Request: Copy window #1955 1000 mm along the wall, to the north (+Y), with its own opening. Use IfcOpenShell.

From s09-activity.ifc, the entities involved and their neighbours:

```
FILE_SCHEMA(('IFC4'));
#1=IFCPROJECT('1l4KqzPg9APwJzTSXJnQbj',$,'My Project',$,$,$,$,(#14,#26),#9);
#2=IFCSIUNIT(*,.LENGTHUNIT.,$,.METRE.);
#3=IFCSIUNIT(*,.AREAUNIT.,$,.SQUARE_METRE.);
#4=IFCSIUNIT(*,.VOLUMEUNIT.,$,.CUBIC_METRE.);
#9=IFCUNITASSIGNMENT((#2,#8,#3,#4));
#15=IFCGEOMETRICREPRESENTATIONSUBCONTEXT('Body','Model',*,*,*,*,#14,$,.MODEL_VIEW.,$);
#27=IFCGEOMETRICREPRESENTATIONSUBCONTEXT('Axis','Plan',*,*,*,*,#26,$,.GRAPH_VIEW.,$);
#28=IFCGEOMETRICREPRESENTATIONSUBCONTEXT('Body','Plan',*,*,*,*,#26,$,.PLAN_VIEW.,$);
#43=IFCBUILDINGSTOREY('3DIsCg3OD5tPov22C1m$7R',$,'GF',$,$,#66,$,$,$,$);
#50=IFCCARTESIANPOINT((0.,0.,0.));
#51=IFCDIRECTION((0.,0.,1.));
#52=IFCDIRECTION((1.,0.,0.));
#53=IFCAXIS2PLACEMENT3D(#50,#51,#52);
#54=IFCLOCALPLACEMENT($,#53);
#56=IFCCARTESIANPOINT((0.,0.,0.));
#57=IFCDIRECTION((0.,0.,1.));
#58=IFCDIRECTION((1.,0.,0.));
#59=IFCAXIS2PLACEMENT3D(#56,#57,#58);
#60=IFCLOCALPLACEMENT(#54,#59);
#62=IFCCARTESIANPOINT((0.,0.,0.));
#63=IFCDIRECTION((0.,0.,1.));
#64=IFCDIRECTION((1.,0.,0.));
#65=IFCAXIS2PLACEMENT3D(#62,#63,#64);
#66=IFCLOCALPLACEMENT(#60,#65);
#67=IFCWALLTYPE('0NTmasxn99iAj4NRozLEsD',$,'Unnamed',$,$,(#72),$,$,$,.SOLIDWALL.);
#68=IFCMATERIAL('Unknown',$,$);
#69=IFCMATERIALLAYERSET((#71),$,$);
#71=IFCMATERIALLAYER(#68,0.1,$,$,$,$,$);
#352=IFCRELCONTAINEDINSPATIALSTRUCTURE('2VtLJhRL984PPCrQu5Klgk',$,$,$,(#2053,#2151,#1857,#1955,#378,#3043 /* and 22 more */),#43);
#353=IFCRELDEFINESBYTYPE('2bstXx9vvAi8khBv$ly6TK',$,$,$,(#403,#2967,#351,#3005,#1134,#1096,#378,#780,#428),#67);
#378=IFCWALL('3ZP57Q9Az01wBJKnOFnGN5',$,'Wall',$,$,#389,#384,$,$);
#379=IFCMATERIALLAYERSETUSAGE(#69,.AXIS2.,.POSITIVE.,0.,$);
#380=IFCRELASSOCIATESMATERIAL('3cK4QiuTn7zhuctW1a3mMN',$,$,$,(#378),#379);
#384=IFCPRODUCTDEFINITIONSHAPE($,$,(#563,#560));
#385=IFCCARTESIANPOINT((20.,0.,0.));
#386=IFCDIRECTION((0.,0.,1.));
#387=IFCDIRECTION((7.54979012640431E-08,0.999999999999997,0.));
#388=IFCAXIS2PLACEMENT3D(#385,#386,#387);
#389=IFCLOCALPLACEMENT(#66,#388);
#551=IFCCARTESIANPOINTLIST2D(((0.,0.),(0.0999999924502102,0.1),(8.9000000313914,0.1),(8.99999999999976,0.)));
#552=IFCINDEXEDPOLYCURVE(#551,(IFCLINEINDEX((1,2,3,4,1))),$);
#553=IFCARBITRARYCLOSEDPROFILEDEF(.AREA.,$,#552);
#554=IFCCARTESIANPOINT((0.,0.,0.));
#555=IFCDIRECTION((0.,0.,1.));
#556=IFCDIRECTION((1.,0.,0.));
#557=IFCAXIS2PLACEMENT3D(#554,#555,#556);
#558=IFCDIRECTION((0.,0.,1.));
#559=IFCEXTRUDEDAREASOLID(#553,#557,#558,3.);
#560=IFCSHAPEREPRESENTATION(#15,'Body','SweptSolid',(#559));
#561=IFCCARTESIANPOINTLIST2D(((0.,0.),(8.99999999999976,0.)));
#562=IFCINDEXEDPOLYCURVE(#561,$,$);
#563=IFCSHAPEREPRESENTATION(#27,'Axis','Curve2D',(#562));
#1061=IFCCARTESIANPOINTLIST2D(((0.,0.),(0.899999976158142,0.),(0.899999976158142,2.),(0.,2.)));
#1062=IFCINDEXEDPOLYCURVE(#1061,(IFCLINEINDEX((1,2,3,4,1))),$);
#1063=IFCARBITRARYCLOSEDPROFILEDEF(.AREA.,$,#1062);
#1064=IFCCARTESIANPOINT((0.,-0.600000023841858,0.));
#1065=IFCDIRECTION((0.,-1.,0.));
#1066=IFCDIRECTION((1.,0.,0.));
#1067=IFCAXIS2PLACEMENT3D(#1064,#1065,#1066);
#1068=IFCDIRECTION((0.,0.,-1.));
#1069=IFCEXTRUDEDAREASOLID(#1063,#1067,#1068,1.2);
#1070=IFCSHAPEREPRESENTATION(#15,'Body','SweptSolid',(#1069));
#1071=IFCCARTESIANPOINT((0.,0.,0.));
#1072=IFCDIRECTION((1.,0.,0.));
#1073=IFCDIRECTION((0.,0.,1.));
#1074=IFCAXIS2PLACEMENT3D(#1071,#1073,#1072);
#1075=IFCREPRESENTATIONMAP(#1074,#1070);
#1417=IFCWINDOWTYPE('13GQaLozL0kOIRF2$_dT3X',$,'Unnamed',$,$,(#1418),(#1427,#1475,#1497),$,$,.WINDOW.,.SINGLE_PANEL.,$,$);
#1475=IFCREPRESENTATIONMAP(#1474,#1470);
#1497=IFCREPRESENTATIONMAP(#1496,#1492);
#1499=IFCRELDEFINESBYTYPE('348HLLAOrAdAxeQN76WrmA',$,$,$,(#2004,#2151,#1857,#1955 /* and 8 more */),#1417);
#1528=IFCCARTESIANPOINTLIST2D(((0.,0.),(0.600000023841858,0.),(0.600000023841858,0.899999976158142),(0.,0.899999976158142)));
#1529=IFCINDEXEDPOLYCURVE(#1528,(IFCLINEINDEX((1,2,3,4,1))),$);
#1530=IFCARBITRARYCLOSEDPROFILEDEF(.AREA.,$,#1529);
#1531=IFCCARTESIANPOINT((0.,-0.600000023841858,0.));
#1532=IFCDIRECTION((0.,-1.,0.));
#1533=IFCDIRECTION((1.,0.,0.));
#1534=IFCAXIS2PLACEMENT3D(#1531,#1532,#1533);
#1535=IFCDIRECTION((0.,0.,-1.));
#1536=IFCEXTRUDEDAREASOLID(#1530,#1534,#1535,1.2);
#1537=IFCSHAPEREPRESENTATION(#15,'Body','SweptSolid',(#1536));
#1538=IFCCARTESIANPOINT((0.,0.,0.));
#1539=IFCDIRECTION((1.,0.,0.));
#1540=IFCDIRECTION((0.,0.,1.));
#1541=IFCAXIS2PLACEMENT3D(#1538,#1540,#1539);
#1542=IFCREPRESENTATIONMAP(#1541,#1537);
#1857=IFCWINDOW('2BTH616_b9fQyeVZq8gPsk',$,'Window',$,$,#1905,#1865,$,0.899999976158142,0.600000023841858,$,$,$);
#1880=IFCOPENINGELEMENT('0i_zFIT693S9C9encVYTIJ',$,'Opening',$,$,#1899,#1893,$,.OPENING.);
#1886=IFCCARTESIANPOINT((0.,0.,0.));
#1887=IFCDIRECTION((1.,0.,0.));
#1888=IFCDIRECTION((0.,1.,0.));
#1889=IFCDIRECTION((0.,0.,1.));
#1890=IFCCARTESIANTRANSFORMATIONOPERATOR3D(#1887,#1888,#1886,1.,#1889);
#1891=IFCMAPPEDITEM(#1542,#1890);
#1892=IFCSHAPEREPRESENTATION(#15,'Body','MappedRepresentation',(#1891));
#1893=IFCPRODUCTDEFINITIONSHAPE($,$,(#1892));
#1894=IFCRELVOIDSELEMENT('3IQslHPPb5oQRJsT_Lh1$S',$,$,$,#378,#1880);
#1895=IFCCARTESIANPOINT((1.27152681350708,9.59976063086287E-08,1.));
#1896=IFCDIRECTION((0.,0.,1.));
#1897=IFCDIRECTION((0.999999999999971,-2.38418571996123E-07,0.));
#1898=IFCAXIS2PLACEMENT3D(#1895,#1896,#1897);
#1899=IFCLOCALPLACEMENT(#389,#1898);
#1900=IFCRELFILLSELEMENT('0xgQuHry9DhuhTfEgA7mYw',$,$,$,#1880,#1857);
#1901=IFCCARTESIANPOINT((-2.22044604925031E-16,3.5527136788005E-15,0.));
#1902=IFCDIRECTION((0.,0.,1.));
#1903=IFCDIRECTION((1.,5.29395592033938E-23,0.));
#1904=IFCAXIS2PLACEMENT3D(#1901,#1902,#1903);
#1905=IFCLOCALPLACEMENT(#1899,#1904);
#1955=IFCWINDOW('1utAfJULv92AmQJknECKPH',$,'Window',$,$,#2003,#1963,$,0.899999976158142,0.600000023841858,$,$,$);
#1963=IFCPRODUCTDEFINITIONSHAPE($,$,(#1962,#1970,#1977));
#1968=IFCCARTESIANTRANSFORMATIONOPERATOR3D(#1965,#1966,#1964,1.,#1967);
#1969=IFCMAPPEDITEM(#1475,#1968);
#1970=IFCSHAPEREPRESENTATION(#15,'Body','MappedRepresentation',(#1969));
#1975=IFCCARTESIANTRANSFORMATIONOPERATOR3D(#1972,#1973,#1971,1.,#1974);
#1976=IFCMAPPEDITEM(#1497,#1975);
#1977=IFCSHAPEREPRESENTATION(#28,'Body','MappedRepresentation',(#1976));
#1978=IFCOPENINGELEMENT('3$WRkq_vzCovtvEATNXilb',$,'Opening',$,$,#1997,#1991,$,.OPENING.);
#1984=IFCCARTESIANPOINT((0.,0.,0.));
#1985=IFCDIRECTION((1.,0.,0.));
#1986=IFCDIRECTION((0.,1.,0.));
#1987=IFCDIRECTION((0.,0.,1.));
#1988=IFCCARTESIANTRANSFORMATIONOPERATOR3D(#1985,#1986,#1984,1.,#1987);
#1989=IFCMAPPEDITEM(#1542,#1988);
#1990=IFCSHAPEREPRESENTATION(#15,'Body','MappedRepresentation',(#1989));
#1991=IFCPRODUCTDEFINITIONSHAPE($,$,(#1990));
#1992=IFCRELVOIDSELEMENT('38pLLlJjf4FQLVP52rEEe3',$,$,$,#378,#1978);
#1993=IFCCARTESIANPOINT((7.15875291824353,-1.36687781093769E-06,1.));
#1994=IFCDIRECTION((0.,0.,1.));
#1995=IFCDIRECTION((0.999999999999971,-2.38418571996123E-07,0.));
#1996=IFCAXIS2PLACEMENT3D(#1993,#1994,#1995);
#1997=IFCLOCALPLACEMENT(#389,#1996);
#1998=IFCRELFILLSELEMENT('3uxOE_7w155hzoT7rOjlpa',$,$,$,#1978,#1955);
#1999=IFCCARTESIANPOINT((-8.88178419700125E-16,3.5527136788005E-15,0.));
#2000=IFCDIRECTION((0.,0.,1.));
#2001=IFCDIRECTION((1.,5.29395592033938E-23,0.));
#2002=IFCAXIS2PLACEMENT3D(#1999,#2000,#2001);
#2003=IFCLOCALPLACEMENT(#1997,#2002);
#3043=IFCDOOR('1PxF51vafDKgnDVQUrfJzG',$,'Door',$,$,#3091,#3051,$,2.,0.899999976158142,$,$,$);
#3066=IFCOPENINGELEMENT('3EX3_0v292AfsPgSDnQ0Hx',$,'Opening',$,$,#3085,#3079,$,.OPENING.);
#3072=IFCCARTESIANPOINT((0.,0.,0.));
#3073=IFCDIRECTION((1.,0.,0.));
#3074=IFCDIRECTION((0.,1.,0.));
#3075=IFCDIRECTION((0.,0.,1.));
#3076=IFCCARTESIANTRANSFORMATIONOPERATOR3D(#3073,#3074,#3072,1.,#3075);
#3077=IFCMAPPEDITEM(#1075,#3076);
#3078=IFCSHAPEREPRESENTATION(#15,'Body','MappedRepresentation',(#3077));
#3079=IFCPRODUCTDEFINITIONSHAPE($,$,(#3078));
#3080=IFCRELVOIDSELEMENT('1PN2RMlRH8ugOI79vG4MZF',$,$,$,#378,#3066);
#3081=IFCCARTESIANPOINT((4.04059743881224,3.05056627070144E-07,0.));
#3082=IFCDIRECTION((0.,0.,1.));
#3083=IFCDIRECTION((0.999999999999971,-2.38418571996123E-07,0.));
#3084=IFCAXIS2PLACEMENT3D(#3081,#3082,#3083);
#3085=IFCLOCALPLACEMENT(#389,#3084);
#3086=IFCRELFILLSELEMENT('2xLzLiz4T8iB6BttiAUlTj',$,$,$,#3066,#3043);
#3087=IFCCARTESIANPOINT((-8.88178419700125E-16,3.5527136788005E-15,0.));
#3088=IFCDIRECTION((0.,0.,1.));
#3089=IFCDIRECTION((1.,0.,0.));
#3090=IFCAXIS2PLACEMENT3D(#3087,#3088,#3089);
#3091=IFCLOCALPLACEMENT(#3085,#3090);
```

```python
import ifcopenshell
import ifcopenshell.api.feature
import ifcopenshell.api.geometry
import ifcopenshell.api.root
import ifcopenshell.geom
import ifcopenshell.util.element
import ifcopenshell.util.placement
import ifcopenshell.util.shape
import ifcopenshell.util.unit

model = ifcopenshell.open("s09-activity.ifc")
unit_scale = ifcopenshell.util.unit.calculate_unit_scale(model)
settings = ifcopenshell.geom.settings()


def volume(element):
    """Net volume in cubic metres, openings subtracted."""
    shape = ifcopenshell.geom.create_shape(settings, element)
    return ifcopenshell.util.shape.get_volume(shape.geometry)


window = model.by_guid("1utAfJULv92AmQJknECKPH")
opening = window.FillsVoids[0].RelatingOpeningElement
wall = opening.VoidsElements[0].RelatingBuildingElement
before = volume(wall)
shift = ifcopenshell.util.placement.get_local_placement(wall.ObjectPlacement)[:3, 0] * 1 / unit_scale

# copy_class copies the void relationship, type, container and properties, but no geometry.
new_opening = ifcopenshell.api.root.copy_class(model, product=opening)
new_opening.Representation = ifcopenshell.util.element.copy_deep(
    model, opening.Representation, exclude=["IfcGeometricRepresentationContext", "IfcRepresentationMap"]
)
new_window = ifcopenshell.api.root.copy_class(model, product=window)
new_window.Representation = ifcopenshell.util.element.copy_deep(
    model, window.Representation, exclude=["IfcGeometricRepresentationContext", "IfcRepresentationMap"]
)
ifcopenshell.api.feature.add_filling(model, opening=new_opening, element=new_window)

for old, new in ((opening, new_opening), (window, new_window)):
    matrix = ifcopenshell.util.placement.get_local_placement(old.ObjectPlacement)
    matrix[:3, 3] += shift
    ifcopenshell.api.geometry.edit_object_placement(model, product=new, matrix=matrix, is_si=False)

after = volume(wall)

print(f"wall volume {before:.3f} -> {after:.3f} m3")

model.write("s09-activity_edited.ifc")
```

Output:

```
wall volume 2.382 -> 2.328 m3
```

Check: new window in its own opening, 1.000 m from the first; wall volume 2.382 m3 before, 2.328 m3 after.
